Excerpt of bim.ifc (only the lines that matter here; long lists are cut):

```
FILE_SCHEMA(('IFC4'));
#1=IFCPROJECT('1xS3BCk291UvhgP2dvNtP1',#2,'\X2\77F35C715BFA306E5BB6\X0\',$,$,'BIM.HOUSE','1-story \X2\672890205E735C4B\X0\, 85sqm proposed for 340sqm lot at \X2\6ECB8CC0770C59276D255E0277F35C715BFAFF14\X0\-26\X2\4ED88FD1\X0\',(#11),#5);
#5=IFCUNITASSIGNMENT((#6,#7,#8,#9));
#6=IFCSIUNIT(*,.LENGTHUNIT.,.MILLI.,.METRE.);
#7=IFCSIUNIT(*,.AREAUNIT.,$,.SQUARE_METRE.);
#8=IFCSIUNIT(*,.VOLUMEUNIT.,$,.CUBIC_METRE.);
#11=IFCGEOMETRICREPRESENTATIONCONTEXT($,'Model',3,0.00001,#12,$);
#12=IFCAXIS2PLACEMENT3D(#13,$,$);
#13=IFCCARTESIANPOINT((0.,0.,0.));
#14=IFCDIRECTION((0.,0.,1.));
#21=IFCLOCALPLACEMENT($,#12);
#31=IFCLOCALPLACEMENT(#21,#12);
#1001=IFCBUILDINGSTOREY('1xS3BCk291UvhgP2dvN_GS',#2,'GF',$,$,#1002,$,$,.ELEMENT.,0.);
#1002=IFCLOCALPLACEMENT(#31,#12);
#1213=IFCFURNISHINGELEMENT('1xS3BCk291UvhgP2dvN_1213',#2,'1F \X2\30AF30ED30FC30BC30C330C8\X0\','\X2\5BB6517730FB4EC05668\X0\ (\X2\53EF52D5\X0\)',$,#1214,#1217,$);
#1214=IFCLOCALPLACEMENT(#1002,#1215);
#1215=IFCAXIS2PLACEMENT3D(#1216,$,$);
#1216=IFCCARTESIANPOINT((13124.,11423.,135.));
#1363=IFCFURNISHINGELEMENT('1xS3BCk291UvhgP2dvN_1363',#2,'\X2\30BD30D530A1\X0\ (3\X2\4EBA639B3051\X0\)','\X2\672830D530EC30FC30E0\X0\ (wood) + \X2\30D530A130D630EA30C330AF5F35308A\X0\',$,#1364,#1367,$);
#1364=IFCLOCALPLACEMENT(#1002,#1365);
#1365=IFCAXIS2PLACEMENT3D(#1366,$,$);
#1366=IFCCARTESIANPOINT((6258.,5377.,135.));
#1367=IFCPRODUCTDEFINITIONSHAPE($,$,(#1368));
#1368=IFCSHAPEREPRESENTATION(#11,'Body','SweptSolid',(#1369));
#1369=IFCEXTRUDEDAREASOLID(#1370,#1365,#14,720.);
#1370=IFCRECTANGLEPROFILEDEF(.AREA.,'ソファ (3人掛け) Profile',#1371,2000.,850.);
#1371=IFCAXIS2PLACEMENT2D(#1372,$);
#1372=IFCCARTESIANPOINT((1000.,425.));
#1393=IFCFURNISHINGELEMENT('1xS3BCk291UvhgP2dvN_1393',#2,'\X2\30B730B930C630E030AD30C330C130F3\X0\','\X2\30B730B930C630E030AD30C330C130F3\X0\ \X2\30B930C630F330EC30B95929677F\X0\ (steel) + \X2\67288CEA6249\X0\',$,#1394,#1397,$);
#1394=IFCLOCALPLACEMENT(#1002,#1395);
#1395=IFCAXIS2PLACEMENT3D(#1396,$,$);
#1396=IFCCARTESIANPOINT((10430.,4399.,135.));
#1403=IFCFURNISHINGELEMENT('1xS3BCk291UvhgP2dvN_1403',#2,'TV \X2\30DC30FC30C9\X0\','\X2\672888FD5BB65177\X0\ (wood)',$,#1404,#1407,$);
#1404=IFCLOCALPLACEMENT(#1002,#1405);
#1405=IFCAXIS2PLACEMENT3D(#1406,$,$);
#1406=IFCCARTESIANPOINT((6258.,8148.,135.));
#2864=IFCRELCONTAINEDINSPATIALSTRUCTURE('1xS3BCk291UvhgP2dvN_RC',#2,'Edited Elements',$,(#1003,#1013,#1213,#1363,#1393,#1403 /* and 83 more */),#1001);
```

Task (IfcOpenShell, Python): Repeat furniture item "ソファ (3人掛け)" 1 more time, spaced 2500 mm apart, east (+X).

```python
import numpy as np
import ifcopenshell
import ifcopenshell.api.geometry
import ifcopenshell.api.root
import ifcopenshell.util.element
import ifcopenshell.util.placement

model = ifcopenshell.open("bim.ifc")


def reuse_history(source, copy):
    """copy_class also copies each property set's owner history, people and application; keep the originals."""
    for rel in copy.IsDefinedBy:
        if rel.is_a("IfcRelDefinesByProperties") and (history := rel.RelatingPropertyDefinition.OwnerHistory):
            rel.RelatingPropertyDefinition.OwnerHistory = source.OwnerHistory
            ifcopenshell.util.element.remove_deep2(model, history)


source = model.by_id(1363)
base = ifcopenshell.util.placement.get_local_placement(source.ObjectPlacement)
step = np.array([1.0, 0.0, 0.0]) * 2500.0

for i in range(1, 2):
    copy = ifcopenshell.api.root.copy_class(model, product=source)
    copy.Representation = ifcopenshell.util.element.copy_deep(
        model, source.Representation, exclude=["IfcGeometricRepresentationContext", "IfcRepresentationMap"]
    )
    reuse_history(source, copy)
    matrix = base.copy()
    matrix[:3, 3] += i * step
    print("added at", matrix[:3, 3].round(3) + 0.0)
    ifcopenshell.api.geometry.edit_object_placement(model, product=copy, matrix=matrix, is_si=False)

model.write("bim_rev.ifc")
```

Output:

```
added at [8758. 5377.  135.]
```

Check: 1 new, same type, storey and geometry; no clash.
